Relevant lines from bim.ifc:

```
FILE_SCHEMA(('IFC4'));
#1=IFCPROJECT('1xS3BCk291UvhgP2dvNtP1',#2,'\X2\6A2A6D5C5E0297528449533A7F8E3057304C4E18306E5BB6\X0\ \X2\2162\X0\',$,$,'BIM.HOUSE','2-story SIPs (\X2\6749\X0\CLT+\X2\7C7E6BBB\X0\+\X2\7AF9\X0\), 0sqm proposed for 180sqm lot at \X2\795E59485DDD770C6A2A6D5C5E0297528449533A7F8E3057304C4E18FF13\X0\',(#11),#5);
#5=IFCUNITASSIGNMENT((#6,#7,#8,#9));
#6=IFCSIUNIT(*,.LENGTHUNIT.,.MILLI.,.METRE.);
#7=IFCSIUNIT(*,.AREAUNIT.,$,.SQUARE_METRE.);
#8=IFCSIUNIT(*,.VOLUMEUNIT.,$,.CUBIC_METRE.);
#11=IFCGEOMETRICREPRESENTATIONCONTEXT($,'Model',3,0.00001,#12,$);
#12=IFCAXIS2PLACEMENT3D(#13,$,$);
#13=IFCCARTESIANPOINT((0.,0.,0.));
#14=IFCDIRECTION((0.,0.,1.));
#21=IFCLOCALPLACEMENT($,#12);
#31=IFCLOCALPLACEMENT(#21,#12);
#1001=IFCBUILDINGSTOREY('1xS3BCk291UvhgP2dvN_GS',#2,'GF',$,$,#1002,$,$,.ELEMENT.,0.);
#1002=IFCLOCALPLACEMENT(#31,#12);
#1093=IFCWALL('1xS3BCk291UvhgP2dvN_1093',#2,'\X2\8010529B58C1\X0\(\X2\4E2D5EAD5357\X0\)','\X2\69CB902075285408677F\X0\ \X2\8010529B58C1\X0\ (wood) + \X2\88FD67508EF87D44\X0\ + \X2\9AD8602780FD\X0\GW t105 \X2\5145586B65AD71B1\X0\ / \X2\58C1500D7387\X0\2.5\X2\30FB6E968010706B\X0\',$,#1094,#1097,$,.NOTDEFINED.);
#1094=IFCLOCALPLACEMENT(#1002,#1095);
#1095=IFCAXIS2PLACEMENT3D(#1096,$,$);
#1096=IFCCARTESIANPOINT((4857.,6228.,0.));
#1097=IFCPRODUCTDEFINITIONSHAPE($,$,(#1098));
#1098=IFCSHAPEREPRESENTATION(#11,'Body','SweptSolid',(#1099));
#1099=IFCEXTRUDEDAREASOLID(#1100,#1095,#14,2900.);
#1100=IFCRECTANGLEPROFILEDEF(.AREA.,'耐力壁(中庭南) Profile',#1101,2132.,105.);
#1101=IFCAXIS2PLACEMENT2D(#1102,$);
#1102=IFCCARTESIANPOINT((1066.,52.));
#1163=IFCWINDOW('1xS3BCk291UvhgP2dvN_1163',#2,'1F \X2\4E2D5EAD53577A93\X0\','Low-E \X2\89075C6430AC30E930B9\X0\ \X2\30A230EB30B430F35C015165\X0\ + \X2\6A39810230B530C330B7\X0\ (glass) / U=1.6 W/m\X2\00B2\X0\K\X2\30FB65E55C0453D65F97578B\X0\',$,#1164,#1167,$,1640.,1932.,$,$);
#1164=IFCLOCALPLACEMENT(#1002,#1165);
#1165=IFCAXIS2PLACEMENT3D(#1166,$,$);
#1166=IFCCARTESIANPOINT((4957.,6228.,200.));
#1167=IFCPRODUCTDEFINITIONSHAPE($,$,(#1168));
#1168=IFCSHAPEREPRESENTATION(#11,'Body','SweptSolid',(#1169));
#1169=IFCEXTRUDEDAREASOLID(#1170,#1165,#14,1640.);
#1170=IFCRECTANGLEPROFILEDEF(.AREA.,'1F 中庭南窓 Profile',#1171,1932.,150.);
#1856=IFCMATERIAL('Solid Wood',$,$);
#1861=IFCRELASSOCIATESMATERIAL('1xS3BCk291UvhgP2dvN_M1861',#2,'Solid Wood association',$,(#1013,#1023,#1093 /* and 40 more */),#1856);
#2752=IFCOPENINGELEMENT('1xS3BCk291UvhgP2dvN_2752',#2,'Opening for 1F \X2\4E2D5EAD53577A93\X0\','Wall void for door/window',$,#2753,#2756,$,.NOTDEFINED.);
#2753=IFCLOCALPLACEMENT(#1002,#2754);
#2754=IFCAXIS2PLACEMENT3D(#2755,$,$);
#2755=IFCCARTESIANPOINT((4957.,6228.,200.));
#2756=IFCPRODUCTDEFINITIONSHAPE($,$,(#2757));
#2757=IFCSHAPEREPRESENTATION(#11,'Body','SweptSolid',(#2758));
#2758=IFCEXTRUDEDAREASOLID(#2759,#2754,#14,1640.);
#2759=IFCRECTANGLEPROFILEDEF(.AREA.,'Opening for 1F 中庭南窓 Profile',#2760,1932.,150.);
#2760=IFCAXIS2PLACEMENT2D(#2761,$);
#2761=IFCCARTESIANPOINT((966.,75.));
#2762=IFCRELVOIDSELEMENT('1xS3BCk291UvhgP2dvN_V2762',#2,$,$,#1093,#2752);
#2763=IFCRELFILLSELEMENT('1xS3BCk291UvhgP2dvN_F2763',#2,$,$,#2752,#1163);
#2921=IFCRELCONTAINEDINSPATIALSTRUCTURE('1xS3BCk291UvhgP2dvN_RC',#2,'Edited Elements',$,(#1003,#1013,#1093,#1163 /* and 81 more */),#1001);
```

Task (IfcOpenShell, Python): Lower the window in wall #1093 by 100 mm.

```python
import numpy as np
import ifcopenshell
import ifcopenshell.api.geometry
import ifcopenshell.util.placement
import ifcopenshell.util.unit

model = ifcopenshell.open("bim.ifc")
unit_scale = ifcopenshell.util.unit.calculate_unit_scale(model)

window = model.by_id(1163)
opening = window.FillsVoids[0].RelatingOpeningElement
dz = -0.1 / unit_scale

shift = np.array([0.0, 0.0, dz])
# The window is not placed relative to its opening, so move both.
for product in (opening, window):
    matrix = ifcopenshell.util.placement.get_local_placement(product.ObjectPlacement)
    matrix[:3, 3] += shift
    ifcopenshell.api.geometry.edit_object_placement(model, product=product, matrix=matrix, is_si=False)

print(f"moved by {dz * unit_scale:+.3f} m")

model.write("bim_edited.ifc")
```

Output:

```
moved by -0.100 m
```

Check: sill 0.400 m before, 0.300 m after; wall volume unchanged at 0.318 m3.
